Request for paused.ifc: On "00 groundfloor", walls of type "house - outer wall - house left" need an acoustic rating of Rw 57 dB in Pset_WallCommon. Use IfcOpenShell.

First a look at what the model holds.

```python
import ifcopenshell
import ifcopenshell.util.element

model = ifcopenshell.open("paused.ifc")
print(model.schema)
storey = next(s for s in model.by_type("IfcBuildingStorey") if s.Name == "00 groundfloor")
walls = [e for e in ifcopenshell.util.element.get_decomposition(storey) if e.is_a("IfcWall")]
seen = {}
for e in walls:
    element_type = ifcopenshell.util.element.get_type(e)
    key = (element_type.Name if element_type != e and element_type else None, ifcopenshell.util.element.get_pset(e, "Pset_WallCommon", "AcousticRating"))
    seen[key] = seen.get(key, 0) + 1
for (name, value), count in sorted(seen.items(), key=str):
    print(count, "x", name, "|", value)
```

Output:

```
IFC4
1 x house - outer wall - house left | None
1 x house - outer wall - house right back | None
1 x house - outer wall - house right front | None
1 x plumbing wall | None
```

```python
import ifcopenshell
import ifcopenshell.api.pset
import ifcopenshell.util.element

model = ifcopenshell.open("paused.ifc")

storey = next(s for s in model.by_type("IfcBuildingStorey") if s.Name == "00 groundfloor")
walls = [e for e in ifcopenshell.util.element.get_decomposition(storey) if e.is_a("IfcWall")]

count = 0
for e in walls:
    element_type = ifcopenshell.util.element.get_type(e)
    if element_type in (None, e) or element_type.Name != "house - outer wall - house left":
        continue
    # add_pset returns the element's existing set when there is one.
    pset = ifcopenshell.api.pset.add_pset(model, product=e, name="Pset_WallCommon")
    ifcopenshell.api.pset.edit_pset(model, pset=pset, properties={"AcousticRating": "Rw 57 dB"})
    count += 1

print(count, "walls updated")

model.write("paused_v2.ifc")
```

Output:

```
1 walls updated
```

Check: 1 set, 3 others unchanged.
